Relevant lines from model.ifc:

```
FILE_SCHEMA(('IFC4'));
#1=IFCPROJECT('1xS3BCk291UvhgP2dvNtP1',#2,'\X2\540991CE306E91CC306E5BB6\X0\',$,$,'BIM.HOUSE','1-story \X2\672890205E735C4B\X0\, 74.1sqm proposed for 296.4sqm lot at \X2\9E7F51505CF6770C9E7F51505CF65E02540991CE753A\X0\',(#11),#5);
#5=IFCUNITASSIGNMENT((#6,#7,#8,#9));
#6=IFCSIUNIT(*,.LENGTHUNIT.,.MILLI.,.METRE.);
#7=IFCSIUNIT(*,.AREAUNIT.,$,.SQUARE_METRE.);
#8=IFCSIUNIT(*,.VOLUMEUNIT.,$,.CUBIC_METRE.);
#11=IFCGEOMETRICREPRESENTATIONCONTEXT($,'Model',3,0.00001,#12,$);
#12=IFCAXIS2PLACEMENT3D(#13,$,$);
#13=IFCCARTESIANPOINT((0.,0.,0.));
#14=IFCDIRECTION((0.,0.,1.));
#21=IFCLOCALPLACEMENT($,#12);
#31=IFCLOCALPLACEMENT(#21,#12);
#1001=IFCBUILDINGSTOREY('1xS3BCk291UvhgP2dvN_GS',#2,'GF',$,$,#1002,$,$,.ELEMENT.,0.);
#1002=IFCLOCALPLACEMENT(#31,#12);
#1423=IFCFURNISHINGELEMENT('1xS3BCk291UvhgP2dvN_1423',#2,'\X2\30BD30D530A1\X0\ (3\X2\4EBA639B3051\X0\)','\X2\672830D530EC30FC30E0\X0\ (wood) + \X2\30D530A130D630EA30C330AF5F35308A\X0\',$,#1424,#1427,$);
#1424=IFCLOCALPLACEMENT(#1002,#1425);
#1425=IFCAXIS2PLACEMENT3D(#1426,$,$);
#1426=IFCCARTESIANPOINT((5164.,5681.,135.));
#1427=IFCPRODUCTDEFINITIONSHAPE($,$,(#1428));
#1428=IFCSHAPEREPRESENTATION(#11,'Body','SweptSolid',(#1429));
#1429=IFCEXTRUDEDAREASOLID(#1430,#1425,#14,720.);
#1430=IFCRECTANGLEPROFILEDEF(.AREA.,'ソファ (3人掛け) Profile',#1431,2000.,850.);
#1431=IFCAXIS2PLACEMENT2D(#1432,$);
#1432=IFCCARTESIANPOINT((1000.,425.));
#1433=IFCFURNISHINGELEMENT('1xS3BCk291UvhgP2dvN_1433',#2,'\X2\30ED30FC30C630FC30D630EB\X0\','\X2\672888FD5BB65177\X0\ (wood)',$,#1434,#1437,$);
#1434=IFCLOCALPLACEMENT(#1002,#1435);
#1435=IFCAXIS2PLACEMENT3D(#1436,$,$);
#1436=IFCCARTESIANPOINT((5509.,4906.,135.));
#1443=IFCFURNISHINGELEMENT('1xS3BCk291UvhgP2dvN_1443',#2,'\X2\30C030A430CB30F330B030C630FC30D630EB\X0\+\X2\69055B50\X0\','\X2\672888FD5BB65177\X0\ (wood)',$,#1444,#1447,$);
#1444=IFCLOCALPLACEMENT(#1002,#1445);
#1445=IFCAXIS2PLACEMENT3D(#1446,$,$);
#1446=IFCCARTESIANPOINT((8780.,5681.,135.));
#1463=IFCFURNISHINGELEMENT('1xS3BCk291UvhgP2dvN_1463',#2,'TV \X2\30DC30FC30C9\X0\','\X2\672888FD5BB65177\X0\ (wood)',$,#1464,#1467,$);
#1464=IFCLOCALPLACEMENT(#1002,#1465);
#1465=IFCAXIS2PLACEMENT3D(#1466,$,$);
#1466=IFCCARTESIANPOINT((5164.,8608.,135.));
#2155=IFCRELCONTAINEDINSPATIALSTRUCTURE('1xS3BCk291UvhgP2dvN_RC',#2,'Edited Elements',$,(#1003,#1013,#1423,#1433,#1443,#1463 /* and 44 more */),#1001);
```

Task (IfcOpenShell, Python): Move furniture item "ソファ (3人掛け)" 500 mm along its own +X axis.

```python
import ifcopenshell
import ifcopenshell.api.geometry
import ifcopenshell.util.placement
import ifcopenshell.util.unit

model = ifcopenshell.open("model.ifc")
unit_scale = ifcopenshell.util.unit.calculate_unit_scale(model)

item = model.by_guid("1xS3BCk291UvhgP2dvN_1423")
matrix = ifcopenshell.util.placement.get_local_placement(item.ObjectPlacement)
matrix[:3, 3] += matrix[:3, 0] * 0.5 / unit_scale
ifcopenshell.api.geometry.edit_object_placement(model, product=item, matrix=matrix, is_si=False)

print(ifcopenshell.util.placement.get_local_placement(item.ObjectPlacement).round(3) + 0.0)

model.write("model-out.ifc")
```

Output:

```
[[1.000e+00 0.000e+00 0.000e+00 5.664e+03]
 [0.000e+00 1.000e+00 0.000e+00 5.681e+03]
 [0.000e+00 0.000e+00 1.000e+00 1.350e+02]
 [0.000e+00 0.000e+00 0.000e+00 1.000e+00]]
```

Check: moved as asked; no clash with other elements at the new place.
